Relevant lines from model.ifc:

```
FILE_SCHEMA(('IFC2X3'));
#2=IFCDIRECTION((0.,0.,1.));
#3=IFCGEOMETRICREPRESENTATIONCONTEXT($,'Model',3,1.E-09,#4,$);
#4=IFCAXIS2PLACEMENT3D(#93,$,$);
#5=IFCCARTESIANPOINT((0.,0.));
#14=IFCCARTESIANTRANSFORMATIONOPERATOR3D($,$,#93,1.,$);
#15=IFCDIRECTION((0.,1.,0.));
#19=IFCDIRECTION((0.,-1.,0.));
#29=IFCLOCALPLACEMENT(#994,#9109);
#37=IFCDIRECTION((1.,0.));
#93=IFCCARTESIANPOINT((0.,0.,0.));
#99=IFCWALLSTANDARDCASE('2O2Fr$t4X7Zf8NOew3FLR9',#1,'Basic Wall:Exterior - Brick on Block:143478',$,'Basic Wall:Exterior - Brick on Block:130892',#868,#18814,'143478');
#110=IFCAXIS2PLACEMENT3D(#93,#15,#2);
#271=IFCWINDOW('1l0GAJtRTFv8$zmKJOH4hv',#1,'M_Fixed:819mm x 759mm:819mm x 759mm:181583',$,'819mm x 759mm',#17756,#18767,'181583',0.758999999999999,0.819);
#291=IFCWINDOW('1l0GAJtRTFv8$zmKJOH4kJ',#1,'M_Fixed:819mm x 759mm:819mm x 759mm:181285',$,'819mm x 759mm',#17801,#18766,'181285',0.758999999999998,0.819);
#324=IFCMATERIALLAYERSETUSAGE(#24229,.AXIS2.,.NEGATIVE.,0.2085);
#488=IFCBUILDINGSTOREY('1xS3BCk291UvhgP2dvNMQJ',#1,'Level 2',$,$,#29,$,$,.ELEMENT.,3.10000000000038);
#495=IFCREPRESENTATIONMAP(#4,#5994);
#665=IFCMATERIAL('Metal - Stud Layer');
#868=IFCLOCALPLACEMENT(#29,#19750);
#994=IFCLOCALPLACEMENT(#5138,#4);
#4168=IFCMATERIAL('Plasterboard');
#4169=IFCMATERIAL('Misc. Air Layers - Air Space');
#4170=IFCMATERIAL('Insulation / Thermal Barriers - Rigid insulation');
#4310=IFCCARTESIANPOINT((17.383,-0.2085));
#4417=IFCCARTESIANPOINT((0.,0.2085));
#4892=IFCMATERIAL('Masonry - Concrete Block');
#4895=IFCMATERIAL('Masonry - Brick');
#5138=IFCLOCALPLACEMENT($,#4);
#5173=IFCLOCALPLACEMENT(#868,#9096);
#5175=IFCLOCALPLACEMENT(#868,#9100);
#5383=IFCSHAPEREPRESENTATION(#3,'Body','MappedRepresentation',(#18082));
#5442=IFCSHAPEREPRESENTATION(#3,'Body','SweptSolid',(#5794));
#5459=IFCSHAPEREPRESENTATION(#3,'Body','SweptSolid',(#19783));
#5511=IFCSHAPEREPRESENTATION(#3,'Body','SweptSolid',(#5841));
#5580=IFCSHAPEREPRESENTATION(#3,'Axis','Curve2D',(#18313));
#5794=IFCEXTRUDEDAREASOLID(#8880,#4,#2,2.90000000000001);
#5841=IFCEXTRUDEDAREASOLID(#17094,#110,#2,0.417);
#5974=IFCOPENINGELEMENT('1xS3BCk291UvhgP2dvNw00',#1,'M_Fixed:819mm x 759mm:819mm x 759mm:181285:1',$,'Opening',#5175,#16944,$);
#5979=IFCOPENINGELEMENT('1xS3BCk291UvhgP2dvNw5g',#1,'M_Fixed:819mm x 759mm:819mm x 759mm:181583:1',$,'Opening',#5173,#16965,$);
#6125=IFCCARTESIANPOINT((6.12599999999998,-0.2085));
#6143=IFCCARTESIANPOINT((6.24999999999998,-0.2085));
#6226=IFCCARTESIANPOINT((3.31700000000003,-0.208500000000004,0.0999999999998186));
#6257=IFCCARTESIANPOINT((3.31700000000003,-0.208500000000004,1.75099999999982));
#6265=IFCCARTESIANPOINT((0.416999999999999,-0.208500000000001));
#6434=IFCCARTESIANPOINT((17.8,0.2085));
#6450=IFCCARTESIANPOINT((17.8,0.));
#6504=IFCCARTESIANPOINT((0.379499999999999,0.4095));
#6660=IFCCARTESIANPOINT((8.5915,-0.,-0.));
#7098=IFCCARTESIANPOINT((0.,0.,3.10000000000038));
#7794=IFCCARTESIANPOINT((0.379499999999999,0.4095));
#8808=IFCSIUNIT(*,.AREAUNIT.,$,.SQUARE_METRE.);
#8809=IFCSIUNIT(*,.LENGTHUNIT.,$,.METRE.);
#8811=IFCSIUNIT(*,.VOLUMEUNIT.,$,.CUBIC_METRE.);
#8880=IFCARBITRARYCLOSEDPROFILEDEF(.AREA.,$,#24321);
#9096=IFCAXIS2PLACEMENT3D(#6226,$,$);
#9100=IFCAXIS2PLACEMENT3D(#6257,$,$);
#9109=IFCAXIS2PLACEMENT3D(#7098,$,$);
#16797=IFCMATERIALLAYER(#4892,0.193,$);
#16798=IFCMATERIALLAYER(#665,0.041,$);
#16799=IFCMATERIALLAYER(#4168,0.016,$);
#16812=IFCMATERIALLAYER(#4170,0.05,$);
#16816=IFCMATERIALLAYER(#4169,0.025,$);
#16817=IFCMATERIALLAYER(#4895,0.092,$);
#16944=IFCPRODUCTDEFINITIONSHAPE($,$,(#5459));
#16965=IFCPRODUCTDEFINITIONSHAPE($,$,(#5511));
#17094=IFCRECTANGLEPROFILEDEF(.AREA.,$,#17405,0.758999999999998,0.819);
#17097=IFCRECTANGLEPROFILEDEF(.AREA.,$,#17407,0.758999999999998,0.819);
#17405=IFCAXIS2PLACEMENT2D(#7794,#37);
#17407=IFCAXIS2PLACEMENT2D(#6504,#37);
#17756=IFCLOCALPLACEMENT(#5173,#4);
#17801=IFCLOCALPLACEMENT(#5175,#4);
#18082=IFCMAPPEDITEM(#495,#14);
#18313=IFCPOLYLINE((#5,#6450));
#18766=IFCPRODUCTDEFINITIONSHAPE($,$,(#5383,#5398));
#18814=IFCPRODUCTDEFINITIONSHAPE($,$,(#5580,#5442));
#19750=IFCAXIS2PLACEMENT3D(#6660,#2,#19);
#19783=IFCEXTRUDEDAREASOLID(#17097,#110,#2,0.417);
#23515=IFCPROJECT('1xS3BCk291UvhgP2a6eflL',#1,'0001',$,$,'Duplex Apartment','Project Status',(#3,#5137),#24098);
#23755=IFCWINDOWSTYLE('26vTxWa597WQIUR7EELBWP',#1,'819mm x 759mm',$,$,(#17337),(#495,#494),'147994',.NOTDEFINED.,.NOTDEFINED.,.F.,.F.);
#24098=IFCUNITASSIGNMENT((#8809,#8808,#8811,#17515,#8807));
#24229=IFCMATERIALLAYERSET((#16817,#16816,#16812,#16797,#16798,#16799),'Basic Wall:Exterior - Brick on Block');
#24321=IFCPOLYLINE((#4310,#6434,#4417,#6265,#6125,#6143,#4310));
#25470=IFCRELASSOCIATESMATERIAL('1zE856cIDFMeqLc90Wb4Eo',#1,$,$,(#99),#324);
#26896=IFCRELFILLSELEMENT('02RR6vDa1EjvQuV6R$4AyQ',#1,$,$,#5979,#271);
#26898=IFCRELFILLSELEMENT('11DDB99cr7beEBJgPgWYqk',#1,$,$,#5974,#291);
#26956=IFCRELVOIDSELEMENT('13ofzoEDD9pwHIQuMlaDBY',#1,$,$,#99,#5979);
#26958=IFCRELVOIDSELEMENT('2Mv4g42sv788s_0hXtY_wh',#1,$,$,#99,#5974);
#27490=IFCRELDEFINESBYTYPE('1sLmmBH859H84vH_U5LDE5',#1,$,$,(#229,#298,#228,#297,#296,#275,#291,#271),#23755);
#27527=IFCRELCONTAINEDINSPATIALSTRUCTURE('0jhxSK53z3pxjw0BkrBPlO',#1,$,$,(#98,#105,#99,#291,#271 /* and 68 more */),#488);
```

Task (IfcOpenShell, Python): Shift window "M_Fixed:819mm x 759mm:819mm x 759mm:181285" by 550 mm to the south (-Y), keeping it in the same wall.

```python
import ifcopenshell
import ifcopenshell.api.geometry
import ifcopenshell.util.placement
import ifcopenshell.util.unit

model = ifcopenshell.open("model.ifc")
unit_scale = ifcopenshell.util.unit.calculate_unit_scale(model)

window = model.by_guid("1l0GAJtRTFv8$zmKJOH4kJ")
opening = window.FillsVoids[0].RelatingOpeningElement
wall = opening.VoidsElements[0].RelatingBuildingElement

wall_matrix = ifcopenshell.util.placement.get_local_placement(wall.ObjectPlacement)
shift = wall_matrix[:3, 0] * 0.55 / unit_scale
before = ifcopenshell.util.placement.get_local_placement(window.ObjectPlacement)[:3, 3].copy()

# The window is placed relative to its opening, so it follows when the opening moves.
matrix = ifcopenshell.util.placement.get_local_placement(opening.ObjectPlacement)
matrix[:3, 3] += shift
ifcopenshell.api.geometry.edit_object_placement(
    model, product=opening, matrix=matrix, is_si=False, should_transform_children=True
)

after = ifcopenshell.util.placement.get_local_placement(window.ObjectPlacement)[:3, 3]
print("window moved by", (after - before).round(3) + 0.0)

model.write("model_v2.ifc")
```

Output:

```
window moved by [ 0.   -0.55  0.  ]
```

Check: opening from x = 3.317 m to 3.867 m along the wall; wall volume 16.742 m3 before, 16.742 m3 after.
